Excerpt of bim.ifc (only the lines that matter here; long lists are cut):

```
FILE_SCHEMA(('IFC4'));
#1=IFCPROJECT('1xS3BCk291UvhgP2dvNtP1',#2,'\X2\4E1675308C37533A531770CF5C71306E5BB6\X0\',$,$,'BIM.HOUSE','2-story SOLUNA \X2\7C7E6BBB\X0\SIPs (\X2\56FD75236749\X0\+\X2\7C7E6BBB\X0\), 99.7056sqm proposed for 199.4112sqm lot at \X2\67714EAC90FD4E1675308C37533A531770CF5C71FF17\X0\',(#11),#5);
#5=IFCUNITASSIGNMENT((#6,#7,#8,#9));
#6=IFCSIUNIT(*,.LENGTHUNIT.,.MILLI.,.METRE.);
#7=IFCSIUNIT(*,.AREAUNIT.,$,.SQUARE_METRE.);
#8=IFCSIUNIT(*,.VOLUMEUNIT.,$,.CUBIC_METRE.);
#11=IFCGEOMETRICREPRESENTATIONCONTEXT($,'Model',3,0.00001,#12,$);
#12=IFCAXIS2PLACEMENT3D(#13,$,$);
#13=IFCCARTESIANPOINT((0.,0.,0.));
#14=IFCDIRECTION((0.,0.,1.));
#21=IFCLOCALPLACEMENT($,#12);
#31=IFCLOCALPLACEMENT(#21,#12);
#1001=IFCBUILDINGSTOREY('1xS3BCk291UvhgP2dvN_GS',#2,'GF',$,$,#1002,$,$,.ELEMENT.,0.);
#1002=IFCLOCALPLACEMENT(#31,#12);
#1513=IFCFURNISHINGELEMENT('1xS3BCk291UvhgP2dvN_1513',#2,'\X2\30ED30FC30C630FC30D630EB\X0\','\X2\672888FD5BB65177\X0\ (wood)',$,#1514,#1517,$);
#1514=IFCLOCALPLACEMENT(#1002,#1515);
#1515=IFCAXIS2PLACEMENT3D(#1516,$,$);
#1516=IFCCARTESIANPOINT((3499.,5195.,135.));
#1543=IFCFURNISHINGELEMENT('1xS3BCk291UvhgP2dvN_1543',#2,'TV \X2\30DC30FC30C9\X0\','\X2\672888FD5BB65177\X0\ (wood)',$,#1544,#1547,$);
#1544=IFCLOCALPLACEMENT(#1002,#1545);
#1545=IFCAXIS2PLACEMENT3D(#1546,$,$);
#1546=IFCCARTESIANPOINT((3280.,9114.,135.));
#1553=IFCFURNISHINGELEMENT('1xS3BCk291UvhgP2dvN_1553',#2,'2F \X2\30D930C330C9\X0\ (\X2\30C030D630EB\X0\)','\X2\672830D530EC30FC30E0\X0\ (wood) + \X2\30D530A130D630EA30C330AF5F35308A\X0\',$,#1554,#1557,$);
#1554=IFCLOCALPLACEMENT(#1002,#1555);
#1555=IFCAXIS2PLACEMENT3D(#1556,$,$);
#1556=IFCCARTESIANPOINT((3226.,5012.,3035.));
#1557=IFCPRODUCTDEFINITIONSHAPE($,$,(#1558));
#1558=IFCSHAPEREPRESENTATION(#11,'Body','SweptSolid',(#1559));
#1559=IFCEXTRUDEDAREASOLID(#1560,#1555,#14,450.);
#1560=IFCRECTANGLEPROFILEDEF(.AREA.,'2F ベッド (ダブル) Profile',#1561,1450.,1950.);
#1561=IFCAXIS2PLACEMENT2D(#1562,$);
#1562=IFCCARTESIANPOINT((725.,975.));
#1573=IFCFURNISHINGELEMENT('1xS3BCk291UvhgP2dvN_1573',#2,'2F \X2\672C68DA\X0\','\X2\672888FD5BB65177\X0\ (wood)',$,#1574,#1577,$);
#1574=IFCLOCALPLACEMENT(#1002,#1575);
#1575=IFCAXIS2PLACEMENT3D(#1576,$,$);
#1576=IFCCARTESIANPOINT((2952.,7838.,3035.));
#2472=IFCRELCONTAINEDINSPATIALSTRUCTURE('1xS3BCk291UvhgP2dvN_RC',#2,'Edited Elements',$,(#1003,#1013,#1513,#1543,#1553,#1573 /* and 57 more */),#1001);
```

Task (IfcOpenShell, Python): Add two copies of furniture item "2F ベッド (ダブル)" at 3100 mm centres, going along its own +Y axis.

```python
import ifcopenshell
import ifcopenshell.api.geometry
import ifcopenshell.api.root
import ifcopenshell.util.element
import ifcopenshell.util.placement

model = ifcopenshell.open("bim.ifc")


def reuse_history(source, copy):
    """copy_class also copies each property set's owner history, people and application; keep the originals."""
    for rel in copy.IsDefinedBy:
        if rel.is_a("IfcRelDefinesByProperties") and (history := rel.RelatingPropertyDefinition.OwnerHistory):
            rel.RelatingPropertyDefinition.OwnerHistory = source.OwnerHistory
            ifcopenshell.util.element.remove_deep2(model, history)


source = model.by_guid("1xS3BCk291UvhgP2dvN_1553")
base = ifcopenshell.util.placement.get_local_placement(source.ObjectPlacement)
step = base[:3, 1] * 3100.0

for i in range(1, 3):
    copy = ifcopenshell.api.root.copy_class(model, product=source)
    copy.Representation = ifcopenshell.util.element.copy_deep(
        model, source.Representation, exclude=["IfcGeometricRepresentationContext", "IfcRepresentationMap"]
    )
    reuse_history(source, copy)
    matrix = base.copy()
    matrix[:3, 3] += i * step
    print("added at", matrix[:3, 3].round(3) + 0.0)
    ifcopenshell.api.geometry.edit_object_placement(model, product=copy, matrix=matrix, is_si=False)

model.write("bim_edited.ifc")
```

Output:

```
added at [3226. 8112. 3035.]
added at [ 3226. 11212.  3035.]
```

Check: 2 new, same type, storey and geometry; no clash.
